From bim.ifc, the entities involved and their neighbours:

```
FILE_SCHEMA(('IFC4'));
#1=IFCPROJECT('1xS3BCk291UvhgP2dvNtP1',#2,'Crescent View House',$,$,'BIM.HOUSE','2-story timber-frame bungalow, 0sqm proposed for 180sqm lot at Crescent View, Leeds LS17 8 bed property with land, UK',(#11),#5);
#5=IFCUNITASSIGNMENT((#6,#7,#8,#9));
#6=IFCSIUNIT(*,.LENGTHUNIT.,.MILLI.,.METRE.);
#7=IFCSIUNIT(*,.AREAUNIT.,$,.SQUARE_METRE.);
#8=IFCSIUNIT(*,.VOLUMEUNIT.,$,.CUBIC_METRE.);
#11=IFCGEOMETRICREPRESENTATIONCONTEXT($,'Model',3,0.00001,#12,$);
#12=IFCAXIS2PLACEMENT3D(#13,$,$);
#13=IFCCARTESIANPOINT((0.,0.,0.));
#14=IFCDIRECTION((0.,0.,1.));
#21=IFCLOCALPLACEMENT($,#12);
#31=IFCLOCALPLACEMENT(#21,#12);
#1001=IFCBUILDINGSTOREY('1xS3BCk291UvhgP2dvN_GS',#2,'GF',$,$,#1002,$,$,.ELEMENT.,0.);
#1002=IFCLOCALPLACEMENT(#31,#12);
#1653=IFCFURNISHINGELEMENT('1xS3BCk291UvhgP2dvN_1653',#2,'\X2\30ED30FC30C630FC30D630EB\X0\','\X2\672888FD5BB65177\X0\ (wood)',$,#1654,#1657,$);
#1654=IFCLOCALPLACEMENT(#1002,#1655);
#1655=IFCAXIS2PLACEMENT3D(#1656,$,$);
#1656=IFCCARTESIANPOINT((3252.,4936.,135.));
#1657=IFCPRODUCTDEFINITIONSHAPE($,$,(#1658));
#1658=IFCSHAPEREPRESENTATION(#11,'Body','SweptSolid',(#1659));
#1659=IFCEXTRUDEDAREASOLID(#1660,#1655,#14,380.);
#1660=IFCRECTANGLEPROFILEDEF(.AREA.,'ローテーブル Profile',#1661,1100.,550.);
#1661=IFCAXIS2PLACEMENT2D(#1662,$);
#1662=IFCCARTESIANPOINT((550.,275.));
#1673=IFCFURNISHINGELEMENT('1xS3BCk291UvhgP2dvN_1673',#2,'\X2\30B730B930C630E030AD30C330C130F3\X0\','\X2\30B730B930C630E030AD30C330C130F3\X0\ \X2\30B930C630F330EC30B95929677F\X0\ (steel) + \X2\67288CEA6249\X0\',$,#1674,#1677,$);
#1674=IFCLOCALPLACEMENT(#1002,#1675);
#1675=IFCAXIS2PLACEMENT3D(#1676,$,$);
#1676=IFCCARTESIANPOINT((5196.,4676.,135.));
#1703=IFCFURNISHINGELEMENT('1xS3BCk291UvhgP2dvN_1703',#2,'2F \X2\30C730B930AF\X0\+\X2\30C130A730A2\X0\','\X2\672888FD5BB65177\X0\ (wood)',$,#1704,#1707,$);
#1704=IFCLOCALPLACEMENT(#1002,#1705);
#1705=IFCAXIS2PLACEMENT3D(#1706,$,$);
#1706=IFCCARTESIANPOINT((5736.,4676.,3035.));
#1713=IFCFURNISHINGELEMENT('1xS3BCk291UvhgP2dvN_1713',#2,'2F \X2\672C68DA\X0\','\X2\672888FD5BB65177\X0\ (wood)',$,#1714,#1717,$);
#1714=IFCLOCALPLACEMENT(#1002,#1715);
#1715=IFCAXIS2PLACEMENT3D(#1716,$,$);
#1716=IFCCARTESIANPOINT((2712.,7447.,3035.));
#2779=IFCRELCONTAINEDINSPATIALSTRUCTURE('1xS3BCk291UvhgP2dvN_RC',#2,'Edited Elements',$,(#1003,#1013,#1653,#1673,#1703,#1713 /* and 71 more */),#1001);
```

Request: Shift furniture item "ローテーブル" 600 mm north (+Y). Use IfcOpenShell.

```python
import ifcopenshell
import ifcopenshell.api.geometry
import ifcopenshell.util.placement
import ifcopenshell.util.unit

model = ifcopenshell.open("bim.ifc")
unit_scale = ifcopenshell.util.unit.calculate_unit_scale(model)

item = model.by_guid("1xS3BCk291UvhgP2dvN_1653")
matrix = ifcopenshell.util.placement.get_local_placement(item.ObjectPlacement)
matrix[1, 3] += 0.6 / unit_scale
ifcopenshell.api.geometry.edit_object_placement(model, product=item, matrix=matrix, is_si=False)

print(ifcopenshell.util.placement.get_local_placement(item.ObjectPlacement).round(3) + 0.0)

model.write("bim_updated.ifc")
```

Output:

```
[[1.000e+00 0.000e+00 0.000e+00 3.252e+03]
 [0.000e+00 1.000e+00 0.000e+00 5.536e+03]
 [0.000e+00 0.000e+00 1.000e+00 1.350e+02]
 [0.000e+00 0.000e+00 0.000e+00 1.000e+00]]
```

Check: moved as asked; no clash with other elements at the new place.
